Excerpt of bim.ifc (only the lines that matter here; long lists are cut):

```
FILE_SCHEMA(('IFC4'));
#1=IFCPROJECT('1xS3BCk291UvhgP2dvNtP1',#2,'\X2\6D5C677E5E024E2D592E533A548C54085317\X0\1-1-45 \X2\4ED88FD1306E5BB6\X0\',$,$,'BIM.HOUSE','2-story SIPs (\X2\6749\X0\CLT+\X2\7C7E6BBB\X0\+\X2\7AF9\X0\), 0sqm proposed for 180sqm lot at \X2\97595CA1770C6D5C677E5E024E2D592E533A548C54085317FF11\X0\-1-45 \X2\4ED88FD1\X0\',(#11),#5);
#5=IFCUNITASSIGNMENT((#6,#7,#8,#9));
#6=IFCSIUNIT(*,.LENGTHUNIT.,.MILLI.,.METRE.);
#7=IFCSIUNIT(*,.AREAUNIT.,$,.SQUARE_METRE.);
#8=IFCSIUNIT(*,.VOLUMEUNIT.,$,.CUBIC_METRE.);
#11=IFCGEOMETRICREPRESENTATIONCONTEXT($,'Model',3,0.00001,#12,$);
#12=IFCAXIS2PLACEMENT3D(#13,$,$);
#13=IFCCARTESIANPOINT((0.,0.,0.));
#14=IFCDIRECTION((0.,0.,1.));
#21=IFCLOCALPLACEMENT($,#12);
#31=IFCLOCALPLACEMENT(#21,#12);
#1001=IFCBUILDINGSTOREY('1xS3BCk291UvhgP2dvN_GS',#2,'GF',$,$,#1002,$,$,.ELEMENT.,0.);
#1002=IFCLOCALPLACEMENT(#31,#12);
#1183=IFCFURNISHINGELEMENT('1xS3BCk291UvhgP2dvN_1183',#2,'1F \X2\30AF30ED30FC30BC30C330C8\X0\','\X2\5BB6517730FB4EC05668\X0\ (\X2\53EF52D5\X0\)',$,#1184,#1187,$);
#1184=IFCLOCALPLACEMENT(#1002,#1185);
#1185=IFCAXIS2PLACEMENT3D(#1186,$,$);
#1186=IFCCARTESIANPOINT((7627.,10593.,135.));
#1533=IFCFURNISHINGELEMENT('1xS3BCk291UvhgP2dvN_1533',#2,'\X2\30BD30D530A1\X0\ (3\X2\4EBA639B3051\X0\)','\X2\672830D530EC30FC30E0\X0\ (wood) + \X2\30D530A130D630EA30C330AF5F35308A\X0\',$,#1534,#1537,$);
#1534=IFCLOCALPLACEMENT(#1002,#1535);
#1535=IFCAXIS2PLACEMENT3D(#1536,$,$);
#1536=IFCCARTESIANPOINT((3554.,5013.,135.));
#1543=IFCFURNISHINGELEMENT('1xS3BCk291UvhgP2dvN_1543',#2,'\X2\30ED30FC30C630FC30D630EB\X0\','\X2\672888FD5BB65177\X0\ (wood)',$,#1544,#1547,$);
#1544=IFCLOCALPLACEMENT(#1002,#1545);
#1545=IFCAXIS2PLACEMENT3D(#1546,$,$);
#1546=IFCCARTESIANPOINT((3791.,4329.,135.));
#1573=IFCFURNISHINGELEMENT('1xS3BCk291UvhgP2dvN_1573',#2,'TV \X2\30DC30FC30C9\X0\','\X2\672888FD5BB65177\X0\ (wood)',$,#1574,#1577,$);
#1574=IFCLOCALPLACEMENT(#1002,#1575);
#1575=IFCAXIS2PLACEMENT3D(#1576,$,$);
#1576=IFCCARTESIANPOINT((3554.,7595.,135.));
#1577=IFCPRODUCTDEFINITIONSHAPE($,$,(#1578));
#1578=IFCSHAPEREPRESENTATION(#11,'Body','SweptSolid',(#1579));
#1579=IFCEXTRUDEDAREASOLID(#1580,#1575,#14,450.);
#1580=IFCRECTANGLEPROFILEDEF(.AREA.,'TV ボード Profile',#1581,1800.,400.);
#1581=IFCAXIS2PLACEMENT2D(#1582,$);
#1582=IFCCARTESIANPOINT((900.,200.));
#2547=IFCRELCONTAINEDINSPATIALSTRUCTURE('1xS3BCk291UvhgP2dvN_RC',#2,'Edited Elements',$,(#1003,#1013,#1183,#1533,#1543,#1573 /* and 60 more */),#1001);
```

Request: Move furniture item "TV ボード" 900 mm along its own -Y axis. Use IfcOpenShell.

```python
import ifcopenshell
import ifcopenshell.api.geometry
import ifcopenshell.util.placement
import ifcopenshell.util.unit

model = ifcopenshell.open("bim.ifc")
unit_scale = ifcopenshell.util.unit.calculate_unit_scale(model)

item = model.by_guid("1xS3BCk291UvhgP2dvN_1573")
matrix = ifcopenshell.util.placement.get_local_placement(item.ObjectPlacement)
matrix[:3, 3] -= matrix[:3, 1] * 0.9 / unit_scale
ifcopenshell.api.geometry.edit_object_placement(model, product=item, matrix=matrix, is_si=False)

print(ifcopenshell.util.placement.get_local_placement(item.ObjectPlacement).round(3) + 0.0)

model.write("bim_updated.ifc")
```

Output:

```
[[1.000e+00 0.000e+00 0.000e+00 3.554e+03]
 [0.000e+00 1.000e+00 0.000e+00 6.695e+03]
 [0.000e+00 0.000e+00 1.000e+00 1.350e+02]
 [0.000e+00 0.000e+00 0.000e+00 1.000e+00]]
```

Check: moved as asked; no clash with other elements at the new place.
